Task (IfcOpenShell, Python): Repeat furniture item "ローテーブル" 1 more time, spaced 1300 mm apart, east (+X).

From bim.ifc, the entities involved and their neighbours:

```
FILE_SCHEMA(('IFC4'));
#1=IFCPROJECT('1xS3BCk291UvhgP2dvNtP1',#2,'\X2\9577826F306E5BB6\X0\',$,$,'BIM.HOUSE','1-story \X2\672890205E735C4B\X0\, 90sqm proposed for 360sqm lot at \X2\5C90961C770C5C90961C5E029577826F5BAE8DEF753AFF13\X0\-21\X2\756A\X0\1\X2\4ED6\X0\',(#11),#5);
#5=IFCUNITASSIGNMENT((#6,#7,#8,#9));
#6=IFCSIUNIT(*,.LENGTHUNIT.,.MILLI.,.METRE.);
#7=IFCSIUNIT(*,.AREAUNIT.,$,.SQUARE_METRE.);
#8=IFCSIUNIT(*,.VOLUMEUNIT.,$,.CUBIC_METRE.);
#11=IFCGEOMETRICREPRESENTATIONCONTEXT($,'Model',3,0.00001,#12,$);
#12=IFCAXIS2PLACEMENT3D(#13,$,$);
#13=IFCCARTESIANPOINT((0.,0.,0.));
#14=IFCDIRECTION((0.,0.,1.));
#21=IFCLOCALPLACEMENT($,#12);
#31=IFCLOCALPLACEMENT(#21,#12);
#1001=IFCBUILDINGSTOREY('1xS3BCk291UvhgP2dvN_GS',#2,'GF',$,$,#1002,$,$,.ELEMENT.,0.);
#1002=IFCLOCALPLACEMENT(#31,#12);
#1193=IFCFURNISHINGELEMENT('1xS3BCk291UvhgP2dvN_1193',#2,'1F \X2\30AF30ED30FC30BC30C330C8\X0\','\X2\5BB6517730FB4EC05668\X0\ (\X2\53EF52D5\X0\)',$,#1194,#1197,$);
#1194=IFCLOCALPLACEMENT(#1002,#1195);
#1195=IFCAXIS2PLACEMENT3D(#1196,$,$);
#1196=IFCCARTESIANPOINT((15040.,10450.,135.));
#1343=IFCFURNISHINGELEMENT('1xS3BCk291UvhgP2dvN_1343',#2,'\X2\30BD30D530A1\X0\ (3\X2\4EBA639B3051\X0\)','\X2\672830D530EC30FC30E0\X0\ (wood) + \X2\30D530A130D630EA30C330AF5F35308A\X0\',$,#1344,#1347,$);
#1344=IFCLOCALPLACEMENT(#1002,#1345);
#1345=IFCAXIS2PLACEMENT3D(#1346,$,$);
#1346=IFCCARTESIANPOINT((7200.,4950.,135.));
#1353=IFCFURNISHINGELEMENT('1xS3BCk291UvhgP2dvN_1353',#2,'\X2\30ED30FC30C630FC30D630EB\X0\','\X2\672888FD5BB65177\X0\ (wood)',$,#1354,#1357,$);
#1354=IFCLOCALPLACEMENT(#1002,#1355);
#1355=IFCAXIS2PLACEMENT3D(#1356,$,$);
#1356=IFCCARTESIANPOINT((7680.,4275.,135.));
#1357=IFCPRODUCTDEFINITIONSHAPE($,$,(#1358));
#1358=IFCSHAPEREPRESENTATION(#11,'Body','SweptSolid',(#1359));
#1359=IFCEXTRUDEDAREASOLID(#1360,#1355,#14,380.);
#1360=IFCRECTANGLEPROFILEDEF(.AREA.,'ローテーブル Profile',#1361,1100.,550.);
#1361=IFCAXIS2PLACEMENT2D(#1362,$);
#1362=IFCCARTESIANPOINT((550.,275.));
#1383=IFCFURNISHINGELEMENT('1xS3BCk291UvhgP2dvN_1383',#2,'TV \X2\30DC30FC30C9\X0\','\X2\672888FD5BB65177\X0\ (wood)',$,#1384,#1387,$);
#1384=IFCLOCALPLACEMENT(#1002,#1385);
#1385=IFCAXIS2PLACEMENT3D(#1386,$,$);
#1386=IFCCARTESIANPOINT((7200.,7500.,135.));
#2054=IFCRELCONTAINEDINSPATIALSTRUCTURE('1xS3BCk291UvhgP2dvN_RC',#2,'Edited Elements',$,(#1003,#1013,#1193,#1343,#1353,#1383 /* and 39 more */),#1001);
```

```python
import numpy as np
import ifcopenshell
import ifcopenshell.api.geometry
import ifcopenshell.api.root
import ifcopenshell.util.element
import ifcopenshell.util.placement
import ifcopenshell.util.unit

model = ifcopenshell.open("bim.ifc")
unit_scale = ifcopenshell.util.unit.calculate_unit_scale(model)


def reuse_history(source, copy):
    """copy_class also copies each property set's owner history, people and application; keep the originals."""
    for rel in copy.IsDefinedBy:
        if rel.is_a("IfcRelDefinesByProperties") and (history := rel.RelatingPropertyDefinition.OwnerHistory):
            rel.RelatingPropertyDefinition.OwnerHistory = source.OwnerHistory
            ifcopenshell.util.element.remove_deep2(model, history)


source = model.by_guid("1xS3BCk291UvhgP2dvN_1353")
base = ifcopenshell.util.placement.get_local_placement(source.ObjectPlacement)
step = np.array([1.0, 0.0, 0.0]) * 1.3 / unit_scale

for i in range(1, 2):
    copy = ifcopenshell.api.root.copy_class(model, product=source)
    copy.Representation = ifcopenshell.util.element.copy_deep(
        model, source.Representation, exclude=["IfcGeometricRepresentationContext", "IfcRepresentationMap"]
    )
    reuse_history(source, copy)
    matrix = base.copy()
    matrix[:3, 3] += i * step
    print("added at", matrix[:3, 3].round(3) + 0.0)
    ifcopenshell.api.geometry.edit_object_placement(model, product=copy, matrix=matrix, is_si=False)

model.write("bim_rev.ifc")
```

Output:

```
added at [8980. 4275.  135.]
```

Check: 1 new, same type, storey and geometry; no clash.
